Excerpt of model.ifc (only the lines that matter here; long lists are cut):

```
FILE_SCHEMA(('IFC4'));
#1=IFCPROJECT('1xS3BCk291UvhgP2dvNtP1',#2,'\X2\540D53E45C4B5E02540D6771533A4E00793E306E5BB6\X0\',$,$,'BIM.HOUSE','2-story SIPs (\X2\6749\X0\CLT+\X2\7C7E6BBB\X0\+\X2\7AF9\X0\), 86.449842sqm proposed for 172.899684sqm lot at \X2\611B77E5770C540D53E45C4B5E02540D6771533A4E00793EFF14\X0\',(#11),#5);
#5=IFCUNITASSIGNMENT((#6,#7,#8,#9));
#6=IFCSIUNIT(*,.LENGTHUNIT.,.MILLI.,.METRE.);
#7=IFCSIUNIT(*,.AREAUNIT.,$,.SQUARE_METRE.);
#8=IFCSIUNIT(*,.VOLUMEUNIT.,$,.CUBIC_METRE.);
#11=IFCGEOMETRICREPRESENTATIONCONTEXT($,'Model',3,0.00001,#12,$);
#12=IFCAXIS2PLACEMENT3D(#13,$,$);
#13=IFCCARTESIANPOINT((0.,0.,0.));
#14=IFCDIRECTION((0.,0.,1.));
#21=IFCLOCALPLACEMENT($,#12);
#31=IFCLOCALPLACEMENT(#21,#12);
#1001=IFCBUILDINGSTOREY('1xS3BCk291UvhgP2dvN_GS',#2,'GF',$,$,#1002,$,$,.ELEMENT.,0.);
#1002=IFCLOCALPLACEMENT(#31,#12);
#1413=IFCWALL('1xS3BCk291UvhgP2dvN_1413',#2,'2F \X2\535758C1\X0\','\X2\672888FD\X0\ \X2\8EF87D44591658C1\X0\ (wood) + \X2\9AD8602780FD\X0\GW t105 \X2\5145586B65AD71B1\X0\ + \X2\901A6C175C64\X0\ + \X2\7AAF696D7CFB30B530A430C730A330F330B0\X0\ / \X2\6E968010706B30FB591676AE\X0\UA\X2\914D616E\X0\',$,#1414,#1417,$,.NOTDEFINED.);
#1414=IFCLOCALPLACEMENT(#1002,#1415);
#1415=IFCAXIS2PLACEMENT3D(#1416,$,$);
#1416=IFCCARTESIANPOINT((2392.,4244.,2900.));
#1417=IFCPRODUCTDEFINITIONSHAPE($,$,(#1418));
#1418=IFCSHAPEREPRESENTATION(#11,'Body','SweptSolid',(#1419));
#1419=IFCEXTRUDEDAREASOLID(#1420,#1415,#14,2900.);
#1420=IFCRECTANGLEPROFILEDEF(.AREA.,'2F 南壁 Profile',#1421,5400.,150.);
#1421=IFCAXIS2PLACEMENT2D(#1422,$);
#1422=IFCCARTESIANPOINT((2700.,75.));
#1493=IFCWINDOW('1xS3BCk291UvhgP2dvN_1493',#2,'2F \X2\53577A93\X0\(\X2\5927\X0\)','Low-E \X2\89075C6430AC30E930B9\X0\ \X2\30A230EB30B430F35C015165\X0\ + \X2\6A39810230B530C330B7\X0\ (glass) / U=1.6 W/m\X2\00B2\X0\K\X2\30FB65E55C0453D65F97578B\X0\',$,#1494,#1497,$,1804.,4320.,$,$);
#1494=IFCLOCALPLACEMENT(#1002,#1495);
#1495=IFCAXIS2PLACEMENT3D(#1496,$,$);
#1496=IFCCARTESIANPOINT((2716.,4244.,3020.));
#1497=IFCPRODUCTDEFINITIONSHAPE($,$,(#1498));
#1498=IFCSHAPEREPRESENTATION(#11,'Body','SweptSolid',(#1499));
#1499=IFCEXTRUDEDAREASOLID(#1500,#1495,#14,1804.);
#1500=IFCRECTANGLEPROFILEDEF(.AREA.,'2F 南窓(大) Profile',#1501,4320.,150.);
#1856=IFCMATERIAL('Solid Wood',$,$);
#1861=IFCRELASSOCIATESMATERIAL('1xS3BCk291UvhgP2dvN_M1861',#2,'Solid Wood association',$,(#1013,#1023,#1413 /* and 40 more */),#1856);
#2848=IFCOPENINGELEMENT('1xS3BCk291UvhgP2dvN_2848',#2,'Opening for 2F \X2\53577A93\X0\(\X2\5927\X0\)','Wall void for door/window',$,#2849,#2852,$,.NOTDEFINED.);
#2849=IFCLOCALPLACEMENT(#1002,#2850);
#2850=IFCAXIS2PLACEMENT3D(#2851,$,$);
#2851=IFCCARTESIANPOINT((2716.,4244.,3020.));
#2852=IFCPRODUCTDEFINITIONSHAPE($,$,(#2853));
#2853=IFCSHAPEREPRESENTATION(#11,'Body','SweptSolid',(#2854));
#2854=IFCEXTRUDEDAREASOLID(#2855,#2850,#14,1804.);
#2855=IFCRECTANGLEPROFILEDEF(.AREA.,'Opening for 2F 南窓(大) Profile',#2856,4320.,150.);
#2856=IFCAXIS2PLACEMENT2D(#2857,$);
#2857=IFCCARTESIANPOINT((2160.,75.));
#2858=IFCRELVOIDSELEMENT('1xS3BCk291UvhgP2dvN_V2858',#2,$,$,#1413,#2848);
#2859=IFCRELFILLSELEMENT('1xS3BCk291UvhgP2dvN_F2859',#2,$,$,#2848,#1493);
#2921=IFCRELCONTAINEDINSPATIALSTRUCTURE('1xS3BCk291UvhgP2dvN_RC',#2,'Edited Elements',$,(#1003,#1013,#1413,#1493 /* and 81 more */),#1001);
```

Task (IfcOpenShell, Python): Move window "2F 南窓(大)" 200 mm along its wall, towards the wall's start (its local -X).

```python
import ifcopenshell
import ifcopenshell.api.geometry
import ifcopenshell.util.placement
import ifcopenshell.util.unit

model = ifcopenshell.open("model.ifc")
unit_scale = ifcopenshell.util.unit.calculate_unit_scale(model)

window = model.by_guid("1xS3BCk291UvhgP2dvN_1493")
opening = window.FillsVoids[0].RelatingOpeningElement
wall = opening.VoidsElements[0].RelatingBuildingElement

wall_matrix = ifcopenshell.util.placement.get_local_placement(wall.ObjectPlacement)
shift = wall_matrix[:3, 0] * -0.2 / unit_scale
before = ifcopenshell.util.placement.get_local_placement(window.ObjectPlacement)[:3, 3].copy()

# The window is not placed relative to its opening, so move both.
for product in (opening, window):
    matrix = ifcopenshell.util.placement.get_local_placement(product.ObjectPlacement)
    matrix[:3, 3] += shift
    ifcopenshell.api.geometry.edit_object_placement(model, product=product, matrix=matrix, is_si=False)

after = ifcopenshell.util.placement.get_local_placement(window.ObjectPlacement)[:3, 3]
print("window moved by", (after - before).round(3) + 0.0)

model.write("model_updated.ifc")
```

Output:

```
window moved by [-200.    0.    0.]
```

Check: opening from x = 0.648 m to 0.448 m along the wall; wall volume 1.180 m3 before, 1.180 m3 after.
